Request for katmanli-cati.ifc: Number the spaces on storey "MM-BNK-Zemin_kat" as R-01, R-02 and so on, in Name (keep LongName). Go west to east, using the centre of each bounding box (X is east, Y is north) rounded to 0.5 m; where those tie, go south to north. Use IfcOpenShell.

First a look at what the model holds.

```python
import ifcopenshell
import ifcopenshell.util.element
import ifcopenshell.util.placement

model = ifcopenshell.open("katmanli-cati.ifc")
print(model.schema)
storey = next(s for s in model.by_type("IfcBuildingStorey") if s.Name == "MM-BNK-Zemin_kat")
spaces = [e for e in ifcopenshell.util.element.get_decomposition(storey) if e.is_a("IfcSpace")]
for e in sorted(spaces, key=lambda e: e.id()):
    origin = ifcopenshell.util.placement.get_local_placement(e.ObjectPlacement)[:3, 3]
    print(e.id(), e.Name, e.LongName, origin.round(2) + 0.0, sep=" | ")
```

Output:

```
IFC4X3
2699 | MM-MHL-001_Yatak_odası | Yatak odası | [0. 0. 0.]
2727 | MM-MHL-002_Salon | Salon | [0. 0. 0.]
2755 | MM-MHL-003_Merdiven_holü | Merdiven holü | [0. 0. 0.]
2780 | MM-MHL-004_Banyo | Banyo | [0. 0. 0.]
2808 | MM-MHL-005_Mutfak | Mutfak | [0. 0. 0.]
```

```python
import ifcopenshell
import ifcopenshell.geom
import ifcopenshell.util.element
import ifcopenshell.util.shape

model = ifcopenshell.open("katmanli-cati.ifc")
settings = ifcopenshell.geom.settings()
settings.set("use-world-coords", True)


def centre(element):
    shape = ifcopenshell.geom.create_shape(settings, element)
    return ifcopenshell.util.shape.get_bbox_centroid(shape.geometry)


storey = next(s for s in model.by_type("IfcBuildingStorey") if s.Name == "MM-BNK-Zemin_kat")
spaces = [e for e in ifcopenshell.util.element.get_decomposition(storey) if e.is_a("IfcSpace")]

# Insertion points can sit at a corner or the storey origin, so sort by the geometry (in metres).
centres = {e: centre(e) for e in spaces}
spaces.sort(key=lambda e: (round(centres[e][0] / 0.5), centres[e][1]))

for i, e in enumerate(spaces, start=1):
    number = f"R-{i:02d}"
    e.Name = number
    print(e.id(), number)

model.write("katmanli-cati_rev.ifc")
```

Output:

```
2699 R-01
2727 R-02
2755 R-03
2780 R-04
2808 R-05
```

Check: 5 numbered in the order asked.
